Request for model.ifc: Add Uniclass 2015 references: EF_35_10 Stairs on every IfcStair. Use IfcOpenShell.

First a look at what the model holds.

```python
import ifcopenshell

model = ifcopenshell.open("model.ifc")
print(model.schema)
print("classifications:", [c.Name for c in model.by_type("IfcClassification")])
for ifc_class in ("IfcDoor", "IfcRoof", "IfcStair", "IfcWall", "IfcWindow"):
    print(ifc_class, len(model.by_type(ifc_class)))
```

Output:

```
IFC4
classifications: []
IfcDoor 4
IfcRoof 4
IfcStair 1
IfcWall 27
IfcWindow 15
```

```python
import ifcopenshell
import ifcopenshell.api.classification

model = ifcopenshell.open("model.ifc")

system = ifcopenshell.api.classification.add_classification(model, classification="Uniclass 2015")

codes = {
    "IfcStair": ("EF_35_10", "Stairs"),
}
for ifc_class, (code, name) in codes.items():
    products = model.by_type(ifc_class)
    ifcopenshell.api.classification.add_reference(
        model, products=products, classification=system, identification=code, name=name
    )
    print(code, len(products))

model.write("model-out.ifc")
```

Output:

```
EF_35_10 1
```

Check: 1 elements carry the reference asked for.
